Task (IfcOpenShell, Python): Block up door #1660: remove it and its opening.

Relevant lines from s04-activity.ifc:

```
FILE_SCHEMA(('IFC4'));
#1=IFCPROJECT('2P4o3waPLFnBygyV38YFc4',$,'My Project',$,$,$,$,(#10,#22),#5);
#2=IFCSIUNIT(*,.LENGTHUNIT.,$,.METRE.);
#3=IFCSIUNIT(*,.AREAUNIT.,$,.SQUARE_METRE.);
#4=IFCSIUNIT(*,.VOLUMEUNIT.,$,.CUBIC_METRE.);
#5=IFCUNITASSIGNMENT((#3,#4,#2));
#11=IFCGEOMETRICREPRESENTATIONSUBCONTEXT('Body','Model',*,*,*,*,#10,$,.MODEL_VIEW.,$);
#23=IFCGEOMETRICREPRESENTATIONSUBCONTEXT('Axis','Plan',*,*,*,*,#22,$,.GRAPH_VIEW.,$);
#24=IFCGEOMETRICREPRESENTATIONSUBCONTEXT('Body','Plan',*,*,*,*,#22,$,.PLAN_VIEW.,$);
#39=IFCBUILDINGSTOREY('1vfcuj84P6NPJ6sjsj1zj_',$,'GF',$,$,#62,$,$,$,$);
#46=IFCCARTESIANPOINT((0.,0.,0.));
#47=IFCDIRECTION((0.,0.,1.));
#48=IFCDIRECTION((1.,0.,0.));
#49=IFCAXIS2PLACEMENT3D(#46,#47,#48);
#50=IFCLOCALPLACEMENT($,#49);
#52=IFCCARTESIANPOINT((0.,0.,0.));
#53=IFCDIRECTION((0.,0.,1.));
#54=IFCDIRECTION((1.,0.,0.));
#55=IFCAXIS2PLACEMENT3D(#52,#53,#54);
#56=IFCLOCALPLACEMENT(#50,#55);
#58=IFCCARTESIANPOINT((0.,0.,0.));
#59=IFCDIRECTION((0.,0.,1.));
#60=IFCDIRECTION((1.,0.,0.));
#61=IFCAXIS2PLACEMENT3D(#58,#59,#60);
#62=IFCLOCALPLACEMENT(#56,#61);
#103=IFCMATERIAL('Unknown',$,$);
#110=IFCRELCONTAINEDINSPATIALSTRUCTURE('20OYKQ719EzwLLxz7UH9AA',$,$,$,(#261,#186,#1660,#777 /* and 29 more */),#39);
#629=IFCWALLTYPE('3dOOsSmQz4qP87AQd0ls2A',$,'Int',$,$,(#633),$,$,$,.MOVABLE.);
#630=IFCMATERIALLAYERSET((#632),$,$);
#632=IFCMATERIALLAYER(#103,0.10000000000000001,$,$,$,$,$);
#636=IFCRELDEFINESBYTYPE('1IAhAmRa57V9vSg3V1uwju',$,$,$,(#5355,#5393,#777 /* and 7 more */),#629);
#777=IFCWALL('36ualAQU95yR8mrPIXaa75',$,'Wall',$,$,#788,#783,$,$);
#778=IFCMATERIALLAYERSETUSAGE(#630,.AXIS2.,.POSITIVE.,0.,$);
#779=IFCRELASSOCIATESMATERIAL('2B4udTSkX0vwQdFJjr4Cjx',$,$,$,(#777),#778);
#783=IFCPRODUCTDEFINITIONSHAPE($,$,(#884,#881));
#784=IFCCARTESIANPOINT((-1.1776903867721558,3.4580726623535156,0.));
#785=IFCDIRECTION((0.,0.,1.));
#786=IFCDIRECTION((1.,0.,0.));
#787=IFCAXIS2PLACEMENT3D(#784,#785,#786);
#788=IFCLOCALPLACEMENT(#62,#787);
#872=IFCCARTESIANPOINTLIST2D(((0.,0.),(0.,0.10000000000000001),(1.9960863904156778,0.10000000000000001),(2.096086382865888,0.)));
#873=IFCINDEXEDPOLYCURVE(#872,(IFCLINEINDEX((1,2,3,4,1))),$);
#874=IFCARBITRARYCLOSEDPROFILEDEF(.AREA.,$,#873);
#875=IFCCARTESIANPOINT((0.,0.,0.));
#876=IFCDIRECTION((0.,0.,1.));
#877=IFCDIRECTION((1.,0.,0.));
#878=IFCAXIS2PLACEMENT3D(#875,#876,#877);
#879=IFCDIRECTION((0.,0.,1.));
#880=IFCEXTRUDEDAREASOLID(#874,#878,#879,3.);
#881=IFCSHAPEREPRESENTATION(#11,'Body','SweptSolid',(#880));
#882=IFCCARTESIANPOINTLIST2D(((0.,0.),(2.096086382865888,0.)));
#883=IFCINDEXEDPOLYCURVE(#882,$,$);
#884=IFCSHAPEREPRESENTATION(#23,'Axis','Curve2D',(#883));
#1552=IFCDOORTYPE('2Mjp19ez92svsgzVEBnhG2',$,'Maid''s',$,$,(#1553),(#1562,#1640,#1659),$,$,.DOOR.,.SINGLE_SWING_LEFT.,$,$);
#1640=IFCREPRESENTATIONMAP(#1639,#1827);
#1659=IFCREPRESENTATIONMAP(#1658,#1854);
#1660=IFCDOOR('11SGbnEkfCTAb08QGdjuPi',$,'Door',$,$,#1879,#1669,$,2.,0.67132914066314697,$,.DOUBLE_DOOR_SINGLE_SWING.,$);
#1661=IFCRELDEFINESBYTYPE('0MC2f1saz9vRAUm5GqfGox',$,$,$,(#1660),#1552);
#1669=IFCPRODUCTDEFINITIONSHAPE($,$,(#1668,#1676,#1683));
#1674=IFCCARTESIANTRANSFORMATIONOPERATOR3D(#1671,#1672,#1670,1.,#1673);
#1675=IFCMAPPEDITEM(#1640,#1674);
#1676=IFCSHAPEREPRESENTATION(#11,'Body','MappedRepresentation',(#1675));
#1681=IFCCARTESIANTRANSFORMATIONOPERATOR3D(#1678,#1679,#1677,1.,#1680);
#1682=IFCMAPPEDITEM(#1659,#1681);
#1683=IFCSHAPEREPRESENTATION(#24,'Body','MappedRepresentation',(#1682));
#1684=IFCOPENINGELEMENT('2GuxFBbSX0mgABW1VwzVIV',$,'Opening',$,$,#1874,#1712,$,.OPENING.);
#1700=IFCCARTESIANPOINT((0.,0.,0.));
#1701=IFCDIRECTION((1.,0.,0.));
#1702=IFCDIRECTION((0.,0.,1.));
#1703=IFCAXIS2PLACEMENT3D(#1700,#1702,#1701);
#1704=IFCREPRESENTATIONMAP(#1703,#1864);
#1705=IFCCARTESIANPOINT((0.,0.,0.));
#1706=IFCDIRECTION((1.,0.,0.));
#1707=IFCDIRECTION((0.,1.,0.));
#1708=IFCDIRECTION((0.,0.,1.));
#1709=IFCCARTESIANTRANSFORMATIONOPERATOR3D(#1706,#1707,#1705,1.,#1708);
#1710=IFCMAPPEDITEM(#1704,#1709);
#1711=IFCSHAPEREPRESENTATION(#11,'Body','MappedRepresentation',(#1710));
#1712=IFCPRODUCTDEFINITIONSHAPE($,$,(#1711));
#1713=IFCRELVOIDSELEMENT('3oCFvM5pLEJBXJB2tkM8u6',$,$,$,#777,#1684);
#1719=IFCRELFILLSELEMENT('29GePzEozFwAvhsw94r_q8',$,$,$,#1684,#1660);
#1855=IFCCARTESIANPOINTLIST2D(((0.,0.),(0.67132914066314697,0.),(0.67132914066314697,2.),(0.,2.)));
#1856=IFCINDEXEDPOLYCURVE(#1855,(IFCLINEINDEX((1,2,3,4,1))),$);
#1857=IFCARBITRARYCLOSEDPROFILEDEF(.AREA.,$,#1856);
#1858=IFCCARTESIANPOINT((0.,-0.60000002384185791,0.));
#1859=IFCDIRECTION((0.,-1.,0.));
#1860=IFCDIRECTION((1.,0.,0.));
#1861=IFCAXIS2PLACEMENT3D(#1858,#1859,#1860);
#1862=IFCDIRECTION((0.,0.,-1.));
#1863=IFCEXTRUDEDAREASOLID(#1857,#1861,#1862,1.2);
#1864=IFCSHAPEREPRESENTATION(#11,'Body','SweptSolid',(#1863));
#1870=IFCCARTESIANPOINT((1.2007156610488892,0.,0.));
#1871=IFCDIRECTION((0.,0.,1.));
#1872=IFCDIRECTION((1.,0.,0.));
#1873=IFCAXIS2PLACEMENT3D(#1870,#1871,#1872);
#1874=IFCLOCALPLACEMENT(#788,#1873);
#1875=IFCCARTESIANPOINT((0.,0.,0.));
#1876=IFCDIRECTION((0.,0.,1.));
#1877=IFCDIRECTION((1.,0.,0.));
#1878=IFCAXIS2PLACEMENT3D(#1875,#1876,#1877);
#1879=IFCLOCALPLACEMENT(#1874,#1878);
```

```python
import ifcopenshell
import ifcopenshell.api.feature
import ifcopenshell.api.root
import ifcopenshell.geom
import ifcopenshell.util.shape

model = ifcopenshell.open("s04-activity.ifc")
settings = ifcopenshell.geom.settings()


def volume(element):
    """Net volume in cubic metres, openings subtracted."""
    shape = ifcopenshell.geom.create_shape(settings, element)
    return ifcopenshell.util.shape.get_volume(shape.geometry)


door = model.by_id(1660)
opening = door.FillsVoids[0].RelatingOpeningElement
wall = opening.VoidsElements[0].RelatingBuildingElement
before = volume(wall)

ifcopenshell.api.root.remove_product(model, product=door)
ifcopenshell.api.feature.remove_feature(model, feature=opening)

after = volume(wall)

print(f"wall volume {before:.3f} -> {after:.3f} m3")

model.write("s04-activity-out.ifc")
```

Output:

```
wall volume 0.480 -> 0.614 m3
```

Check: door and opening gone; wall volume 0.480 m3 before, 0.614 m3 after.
